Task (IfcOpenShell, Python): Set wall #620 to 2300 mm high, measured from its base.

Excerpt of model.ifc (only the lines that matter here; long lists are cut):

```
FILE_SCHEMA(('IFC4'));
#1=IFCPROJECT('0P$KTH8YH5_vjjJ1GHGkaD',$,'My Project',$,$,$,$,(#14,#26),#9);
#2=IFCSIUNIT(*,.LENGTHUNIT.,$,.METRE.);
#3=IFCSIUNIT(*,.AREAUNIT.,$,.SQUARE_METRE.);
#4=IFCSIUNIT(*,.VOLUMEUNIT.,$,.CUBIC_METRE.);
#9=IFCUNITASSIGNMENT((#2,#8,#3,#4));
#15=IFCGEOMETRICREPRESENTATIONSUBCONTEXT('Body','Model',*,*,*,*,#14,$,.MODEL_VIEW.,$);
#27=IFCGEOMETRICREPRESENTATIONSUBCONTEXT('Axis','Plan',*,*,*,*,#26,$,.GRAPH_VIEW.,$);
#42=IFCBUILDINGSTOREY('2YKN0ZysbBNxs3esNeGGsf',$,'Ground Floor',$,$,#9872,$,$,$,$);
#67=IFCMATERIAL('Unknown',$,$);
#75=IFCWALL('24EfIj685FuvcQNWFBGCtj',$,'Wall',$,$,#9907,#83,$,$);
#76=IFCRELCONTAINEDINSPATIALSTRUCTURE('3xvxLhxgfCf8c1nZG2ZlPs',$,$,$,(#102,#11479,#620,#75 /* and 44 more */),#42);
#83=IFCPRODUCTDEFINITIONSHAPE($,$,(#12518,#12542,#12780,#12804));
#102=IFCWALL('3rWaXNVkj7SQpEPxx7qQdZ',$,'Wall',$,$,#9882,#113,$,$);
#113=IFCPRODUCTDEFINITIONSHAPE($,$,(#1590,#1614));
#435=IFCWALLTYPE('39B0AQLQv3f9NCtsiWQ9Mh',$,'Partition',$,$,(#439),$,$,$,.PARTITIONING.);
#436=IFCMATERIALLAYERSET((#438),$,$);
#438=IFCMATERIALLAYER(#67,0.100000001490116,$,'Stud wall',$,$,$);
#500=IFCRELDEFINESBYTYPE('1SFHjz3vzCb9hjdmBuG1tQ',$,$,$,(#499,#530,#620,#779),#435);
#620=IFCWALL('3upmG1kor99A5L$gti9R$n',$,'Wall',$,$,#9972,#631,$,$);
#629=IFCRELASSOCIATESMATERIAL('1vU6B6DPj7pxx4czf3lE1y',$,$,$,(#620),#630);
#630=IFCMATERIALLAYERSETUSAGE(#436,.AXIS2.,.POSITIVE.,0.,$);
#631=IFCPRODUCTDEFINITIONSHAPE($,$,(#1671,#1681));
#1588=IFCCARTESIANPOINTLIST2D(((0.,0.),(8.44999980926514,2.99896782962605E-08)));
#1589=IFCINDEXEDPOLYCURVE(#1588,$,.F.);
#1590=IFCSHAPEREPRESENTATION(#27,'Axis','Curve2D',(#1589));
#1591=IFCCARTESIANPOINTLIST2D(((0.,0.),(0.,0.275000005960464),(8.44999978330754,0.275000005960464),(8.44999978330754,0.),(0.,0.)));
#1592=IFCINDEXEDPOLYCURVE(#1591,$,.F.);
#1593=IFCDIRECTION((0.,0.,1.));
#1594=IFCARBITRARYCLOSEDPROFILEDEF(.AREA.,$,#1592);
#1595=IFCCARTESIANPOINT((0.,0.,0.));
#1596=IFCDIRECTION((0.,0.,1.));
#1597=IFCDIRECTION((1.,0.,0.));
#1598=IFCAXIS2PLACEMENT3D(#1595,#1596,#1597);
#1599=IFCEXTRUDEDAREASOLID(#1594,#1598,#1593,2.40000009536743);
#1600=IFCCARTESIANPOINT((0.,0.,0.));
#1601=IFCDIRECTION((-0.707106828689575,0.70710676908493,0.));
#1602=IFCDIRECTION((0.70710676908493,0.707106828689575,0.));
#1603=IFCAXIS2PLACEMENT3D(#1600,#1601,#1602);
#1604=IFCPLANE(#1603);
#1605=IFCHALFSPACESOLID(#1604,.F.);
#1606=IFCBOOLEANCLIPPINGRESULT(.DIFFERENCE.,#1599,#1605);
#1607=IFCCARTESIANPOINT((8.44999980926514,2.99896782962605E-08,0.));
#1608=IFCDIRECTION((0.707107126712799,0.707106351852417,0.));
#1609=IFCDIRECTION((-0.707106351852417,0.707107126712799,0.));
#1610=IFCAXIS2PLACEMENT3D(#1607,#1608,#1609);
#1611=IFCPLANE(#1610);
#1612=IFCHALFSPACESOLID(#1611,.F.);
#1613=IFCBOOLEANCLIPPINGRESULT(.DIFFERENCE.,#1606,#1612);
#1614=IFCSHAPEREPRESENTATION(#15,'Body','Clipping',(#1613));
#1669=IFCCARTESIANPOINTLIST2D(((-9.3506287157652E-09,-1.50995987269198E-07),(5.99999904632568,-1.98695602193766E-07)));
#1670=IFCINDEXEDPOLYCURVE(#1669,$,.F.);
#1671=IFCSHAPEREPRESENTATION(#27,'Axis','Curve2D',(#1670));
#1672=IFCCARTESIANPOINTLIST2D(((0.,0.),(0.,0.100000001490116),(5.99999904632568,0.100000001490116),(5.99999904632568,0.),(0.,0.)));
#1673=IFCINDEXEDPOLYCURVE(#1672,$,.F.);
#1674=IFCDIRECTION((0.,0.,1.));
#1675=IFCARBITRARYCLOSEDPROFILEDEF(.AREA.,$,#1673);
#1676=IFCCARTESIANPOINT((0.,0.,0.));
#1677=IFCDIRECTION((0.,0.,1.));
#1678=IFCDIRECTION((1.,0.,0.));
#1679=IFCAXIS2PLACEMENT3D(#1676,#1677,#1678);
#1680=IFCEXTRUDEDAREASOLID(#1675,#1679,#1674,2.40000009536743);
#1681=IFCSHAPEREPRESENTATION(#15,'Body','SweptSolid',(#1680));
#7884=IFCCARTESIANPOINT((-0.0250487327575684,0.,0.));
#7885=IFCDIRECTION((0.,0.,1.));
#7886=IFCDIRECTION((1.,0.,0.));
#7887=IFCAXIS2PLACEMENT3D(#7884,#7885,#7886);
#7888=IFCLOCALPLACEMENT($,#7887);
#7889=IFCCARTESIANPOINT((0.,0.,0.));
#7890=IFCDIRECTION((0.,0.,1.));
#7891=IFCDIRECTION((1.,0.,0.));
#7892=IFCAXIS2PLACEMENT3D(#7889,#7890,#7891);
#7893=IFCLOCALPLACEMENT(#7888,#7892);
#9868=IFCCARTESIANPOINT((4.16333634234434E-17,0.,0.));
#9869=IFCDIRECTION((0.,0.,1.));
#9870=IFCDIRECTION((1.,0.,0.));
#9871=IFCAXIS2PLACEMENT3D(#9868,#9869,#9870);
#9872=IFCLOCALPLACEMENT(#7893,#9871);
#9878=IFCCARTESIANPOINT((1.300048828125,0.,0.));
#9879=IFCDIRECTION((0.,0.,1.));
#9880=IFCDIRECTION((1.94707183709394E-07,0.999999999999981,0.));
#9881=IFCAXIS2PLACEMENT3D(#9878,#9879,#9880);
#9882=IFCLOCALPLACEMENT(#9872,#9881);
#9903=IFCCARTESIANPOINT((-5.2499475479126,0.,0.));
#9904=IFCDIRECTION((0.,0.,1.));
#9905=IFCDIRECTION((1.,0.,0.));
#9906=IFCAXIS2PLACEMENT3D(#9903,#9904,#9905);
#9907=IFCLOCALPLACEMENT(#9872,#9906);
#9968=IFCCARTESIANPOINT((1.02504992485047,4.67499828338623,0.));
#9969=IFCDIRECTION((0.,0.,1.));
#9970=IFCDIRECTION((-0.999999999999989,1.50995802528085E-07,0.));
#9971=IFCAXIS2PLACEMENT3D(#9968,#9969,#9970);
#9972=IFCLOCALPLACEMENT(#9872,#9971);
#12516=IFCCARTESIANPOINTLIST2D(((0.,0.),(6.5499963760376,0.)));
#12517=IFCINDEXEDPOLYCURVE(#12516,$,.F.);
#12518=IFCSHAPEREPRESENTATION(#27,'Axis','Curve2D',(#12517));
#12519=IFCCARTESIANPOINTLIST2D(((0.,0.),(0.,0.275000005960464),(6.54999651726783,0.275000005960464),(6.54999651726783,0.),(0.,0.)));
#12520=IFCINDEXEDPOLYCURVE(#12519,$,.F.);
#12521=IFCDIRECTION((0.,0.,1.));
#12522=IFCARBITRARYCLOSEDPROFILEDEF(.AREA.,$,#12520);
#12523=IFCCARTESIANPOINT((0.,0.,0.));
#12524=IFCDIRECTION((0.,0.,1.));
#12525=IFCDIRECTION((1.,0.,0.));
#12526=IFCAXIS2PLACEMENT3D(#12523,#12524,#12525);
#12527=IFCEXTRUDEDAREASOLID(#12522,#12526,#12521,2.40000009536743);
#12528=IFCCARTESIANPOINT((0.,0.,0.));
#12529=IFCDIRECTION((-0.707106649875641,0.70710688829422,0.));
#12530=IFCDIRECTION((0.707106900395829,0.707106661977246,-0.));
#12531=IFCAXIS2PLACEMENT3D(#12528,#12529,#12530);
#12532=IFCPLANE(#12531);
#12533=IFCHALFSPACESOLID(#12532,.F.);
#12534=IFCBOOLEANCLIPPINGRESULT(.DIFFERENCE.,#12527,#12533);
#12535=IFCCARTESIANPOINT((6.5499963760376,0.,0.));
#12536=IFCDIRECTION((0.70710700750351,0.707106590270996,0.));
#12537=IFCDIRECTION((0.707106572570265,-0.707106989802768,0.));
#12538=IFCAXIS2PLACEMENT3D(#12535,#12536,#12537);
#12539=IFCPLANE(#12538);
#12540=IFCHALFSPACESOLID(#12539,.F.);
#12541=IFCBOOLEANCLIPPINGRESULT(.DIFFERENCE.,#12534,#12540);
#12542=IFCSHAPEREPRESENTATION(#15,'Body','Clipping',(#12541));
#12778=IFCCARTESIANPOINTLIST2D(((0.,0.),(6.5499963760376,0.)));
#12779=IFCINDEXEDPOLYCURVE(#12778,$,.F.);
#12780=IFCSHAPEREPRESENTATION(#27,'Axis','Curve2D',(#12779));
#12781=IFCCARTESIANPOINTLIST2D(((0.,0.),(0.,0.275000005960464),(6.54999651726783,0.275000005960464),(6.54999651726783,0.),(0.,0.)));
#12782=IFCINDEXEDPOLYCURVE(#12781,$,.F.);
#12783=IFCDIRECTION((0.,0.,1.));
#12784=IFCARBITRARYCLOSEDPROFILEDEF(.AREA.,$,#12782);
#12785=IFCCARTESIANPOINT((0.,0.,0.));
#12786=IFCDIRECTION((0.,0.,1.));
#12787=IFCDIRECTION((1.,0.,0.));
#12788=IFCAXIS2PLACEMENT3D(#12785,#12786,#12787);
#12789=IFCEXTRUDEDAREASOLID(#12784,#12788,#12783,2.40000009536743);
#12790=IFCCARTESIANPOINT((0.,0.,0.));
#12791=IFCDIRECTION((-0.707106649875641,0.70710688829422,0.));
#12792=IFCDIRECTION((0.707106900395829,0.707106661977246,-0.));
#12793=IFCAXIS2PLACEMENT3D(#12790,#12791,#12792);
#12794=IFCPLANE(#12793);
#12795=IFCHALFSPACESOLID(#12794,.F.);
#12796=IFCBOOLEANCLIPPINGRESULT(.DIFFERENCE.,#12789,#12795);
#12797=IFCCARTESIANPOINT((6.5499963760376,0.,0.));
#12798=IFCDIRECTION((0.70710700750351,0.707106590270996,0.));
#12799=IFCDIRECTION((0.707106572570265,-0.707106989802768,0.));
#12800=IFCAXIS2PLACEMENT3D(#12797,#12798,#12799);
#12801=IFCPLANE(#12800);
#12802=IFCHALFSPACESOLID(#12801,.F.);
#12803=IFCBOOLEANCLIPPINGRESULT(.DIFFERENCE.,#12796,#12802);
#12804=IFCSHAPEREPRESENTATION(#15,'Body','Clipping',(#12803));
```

```python
import ifcopenshell
import ifcopenshell.geom
import ifcopenshell.util.representation
import ifcopenshell.util.shape

model = ifcopenshell.open("model.ifc")
settings = ifcopenshell.geom.settings()


def volume(element):
    """Net volume in cubic metres, openings subtracted."""
    shape = ifcopenshell.geom.create_shape(settings, element)
    return ifcopenshell.util.shape.get_volume(shape.geometry)


wall = model.by_guid("3upmG1kor99A5L$gti9R$n")
before = volume(wall)

body = ifcopenshell.util.representation.get_representation(wall, "Model", "Body")
solid = body.Items[0]
old_height = solid.Depth
solid.Depth = 2.3
after = volume(wall)

print(f"height {old_height:g} -> {solid.Depth:g}, volume {before:.3f} -> {after:.3f} m3")

model.write("model_edited.ifc")
```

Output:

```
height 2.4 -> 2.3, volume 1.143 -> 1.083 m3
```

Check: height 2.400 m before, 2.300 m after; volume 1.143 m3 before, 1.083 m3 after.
